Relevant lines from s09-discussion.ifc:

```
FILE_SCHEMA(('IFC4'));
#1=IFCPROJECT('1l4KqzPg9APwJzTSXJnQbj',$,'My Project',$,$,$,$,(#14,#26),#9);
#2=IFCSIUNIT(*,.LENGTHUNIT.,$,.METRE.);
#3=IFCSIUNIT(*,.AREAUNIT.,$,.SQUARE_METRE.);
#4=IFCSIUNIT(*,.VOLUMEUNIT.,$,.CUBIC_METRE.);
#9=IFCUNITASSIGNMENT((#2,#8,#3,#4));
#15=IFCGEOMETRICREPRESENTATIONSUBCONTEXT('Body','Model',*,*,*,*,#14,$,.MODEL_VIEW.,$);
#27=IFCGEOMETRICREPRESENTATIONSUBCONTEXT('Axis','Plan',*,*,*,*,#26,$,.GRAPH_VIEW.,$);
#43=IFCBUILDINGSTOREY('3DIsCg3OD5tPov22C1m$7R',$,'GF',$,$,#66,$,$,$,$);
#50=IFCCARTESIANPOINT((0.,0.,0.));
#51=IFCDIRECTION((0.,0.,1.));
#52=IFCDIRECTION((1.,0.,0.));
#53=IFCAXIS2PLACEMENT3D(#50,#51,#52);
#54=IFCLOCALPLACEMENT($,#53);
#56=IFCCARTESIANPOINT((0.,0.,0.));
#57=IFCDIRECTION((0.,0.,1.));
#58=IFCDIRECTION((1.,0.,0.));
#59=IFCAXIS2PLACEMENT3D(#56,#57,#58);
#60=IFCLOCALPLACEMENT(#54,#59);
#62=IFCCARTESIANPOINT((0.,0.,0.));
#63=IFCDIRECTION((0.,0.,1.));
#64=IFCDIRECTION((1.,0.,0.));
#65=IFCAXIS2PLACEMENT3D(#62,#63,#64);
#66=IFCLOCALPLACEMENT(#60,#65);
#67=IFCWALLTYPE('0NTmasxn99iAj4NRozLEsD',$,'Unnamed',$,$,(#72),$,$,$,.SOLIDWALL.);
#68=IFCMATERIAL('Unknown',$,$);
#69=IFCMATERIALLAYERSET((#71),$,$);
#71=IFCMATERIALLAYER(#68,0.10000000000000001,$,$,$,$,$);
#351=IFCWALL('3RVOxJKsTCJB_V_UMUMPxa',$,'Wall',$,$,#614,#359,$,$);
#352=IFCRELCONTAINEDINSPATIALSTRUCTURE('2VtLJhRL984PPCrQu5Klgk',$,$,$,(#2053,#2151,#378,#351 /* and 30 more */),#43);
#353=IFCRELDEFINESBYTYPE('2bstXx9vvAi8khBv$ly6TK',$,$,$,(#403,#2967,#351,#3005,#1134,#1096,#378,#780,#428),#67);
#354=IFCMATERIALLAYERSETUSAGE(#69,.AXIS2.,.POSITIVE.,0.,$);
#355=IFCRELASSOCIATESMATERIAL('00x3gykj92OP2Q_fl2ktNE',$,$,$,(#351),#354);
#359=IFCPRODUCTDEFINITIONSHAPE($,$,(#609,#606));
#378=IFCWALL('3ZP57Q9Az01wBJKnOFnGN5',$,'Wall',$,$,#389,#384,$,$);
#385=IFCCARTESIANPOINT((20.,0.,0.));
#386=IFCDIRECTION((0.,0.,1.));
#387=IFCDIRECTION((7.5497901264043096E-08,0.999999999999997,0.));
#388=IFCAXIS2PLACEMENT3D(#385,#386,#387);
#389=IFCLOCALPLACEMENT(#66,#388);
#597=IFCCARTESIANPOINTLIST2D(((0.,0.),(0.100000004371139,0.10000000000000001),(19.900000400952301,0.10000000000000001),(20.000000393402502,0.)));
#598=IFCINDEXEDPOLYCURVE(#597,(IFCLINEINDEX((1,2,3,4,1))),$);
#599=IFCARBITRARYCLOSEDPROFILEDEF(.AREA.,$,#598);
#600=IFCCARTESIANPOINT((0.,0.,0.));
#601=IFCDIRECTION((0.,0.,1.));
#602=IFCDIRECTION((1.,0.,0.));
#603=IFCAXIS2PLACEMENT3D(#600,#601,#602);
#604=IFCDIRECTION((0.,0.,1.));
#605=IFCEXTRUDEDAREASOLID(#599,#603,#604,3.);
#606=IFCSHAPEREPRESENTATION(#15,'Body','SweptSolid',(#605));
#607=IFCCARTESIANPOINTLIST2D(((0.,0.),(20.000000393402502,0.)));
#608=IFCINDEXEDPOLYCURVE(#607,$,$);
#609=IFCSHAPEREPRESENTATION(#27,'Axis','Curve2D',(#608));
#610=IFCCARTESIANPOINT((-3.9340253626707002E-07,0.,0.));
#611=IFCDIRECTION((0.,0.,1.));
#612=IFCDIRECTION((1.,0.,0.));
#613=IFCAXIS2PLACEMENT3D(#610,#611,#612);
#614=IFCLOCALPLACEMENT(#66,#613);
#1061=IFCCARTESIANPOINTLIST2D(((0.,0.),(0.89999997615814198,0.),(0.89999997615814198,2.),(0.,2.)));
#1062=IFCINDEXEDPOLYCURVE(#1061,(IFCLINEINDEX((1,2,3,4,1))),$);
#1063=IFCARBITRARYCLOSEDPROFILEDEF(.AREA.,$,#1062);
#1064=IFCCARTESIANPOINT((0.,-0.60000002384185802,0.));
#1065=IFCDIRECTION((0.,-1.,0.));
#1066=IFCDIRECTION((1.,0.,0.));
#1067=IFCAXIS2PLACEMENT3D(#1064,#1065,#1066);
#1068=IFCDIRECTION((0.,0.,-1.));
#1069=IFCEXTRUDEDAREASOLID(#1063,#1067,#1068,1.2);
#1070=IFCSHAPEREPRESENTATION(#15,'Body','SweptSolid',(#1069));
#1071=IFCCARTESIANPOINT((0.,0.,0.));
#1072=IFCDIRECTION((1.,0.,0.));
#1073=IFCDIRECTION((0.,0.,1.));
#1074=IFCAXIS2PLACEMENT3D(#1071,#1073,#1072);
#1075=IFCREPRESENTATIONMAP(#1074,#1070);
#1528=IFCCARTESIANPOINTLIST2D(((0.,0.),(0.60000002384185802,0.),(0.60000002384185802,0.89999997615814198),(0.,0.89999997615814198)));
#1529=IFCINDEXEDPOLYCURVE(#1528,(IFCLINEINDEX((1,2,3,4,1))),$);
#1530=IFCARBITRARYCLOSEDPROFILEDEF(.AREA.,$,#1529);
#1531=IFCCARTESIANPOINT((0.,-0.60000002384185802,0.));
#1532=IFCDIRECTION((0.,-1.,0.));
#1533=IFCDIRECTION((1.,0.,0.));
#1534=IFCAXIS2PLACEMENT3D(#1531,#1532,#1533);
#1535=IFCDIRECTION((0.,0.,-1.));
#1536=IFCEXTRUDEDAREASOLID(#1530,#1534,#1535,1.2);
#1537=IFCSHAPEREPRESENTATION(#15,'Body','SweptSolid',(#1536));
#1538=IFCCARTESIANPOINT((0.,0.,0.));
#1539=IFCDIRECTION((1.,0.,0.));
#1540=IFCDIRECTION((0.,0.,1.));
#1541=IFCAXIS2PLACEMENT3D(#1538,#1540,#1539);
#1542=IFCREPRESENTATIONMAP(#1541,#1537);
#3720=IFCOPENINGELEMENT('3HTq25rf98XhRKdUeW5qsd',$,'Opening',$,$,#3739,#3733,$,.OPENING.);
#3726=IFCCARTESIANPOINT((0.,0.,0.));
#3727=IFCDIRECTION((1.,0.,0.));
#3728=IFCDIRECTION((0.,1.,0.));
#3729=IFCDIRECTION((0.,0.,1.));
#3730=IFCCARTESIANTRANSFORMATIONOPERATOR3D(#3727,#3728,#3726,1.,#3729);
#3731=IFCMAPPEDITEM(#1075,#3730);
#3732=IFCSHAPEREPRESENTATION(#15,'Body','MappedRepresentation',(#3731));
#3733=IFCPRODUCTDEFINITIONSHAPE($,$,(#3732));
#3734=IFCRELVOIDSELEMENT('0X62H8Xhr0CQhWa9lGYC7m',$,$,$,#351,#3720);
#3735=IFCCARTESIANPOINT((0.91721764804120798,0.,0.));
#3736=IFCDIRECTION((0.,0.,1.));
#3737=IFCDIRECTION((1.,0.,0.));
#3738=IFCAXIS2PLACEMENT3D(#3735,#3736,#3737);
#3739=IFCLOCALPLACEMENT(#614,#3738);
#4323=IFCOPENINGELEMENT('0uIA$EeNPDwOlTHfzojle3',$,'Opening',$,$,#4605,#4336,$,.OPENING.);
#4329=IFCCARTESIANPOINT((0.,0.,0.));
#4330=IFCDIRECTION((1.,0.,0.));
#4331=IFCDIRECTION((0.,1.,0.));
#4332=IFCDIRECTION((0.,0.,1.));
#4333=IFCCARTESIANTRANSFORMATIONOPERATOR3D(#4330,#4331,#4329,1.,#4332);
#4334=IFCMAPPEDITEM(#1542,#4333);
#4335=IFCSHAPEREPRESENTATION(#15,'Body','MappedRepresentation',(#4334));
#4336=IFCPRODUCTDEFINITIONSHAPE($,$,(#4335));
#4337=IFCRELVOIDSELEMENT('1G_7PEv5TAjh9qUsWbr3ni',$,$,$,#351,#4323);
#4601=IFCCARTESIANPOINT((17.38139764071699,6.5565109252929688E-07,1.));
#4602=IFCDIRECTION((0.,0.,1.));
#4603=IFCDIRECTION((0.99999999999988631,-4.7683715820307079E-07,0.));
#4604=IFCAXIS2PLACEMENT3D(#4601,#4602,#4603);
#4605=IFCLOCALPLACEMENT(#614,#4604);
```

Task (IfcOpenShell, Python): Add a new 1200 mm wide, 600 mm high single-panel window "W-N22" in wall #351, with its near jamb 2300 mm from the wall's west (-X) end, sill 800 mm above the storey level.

```python
import numpy as np
import ifcopenshell
import ifcopenshell.api.feature
import ifcopenshell.api.geometry
import ifcopenshell.api.root
import ifcopenshell.api.spatial
import ifcopenshell.geom
import ifcopenshell.util.element
import ifcopenshell.util.placement
import ifcopenshell.util.representation
import ifcopenshell.util.shape
import ifcopenshell.util.unit

model = ifcopenshell.open("s09-discussion.ifc")
unit_scale = ifcopenshell.util.unit.calculate_unit_scale(model)
settings = ifcopenshell.geom.settings()


def volume(element):
    """Net volume in cubic metres, openings subtracted."""
    shape = ifcopenshell.geom.create_shape(settings, element)
    return ifcopenshell.util.shape.get_volume(shape.geometry)


wall = model.by_id(351)
storey = ifcopenshell.util.element.get_container(wall, ifc_class="IfcBuildingStorey")
context = ifcopenshell.util.representation.get_context(model, "Model", "Body", "MODEL_VIEW")
before = volume(wall)

width, height, from_end, sill = 1.2, 0.6, 2.3, 0.8  # metres

# The wall runs along its own X axis, and the end named is its -X end.
wall_shape = ifcopenshell.geom.create_shape(settings, wall)
x, y, z = ifcopenshell.util.shape.get_vertices(wall_shape.geometry).T
start = x.min() + from_end
face, thickness = float(y.min()), float(y.max() - y.min())
wall_matrix = ifcopenshell.util.placement.get_local_placement(wall.ObjectPlacement)
level = ifcopenshell.util.placement.get_local_placement(storey.ObjectPlacement)[2, 3]


def in_wall(x, y):
    """Placement at x, y metres in the wall's axes, at sill height."""
    matrix = wall_matrix.copy()
    matrix[:, 3] = wall_matrix @ np.array([x / unit_scale, y / unit_scale, 0.0, 1.0])
    matrix[2, 3] = level + sill / unit_scale
    return matrix


# Opening: a box that overshoots both wall faces by 50 mm.
opening = ifcopenshell.api.root.create_entity(model, ifc_class="IfcOpeningElement", predefined_type="OPENING")
box = ifcopenshell.api.geometry.add_wall_representation(
    model, context=context, length=width, height=height, thickness=thickness + 0.1
)
ifcopenshell.api.geometry.assign_representation(model, product=opening, representation=box)
ifcopenshell.api.geometry.edit_object_placement(model, product=opening, matrix=in_wall(start, face - 0.05), is_si=False)
ifcopenshell.api.feature.add_feature(model, feature=opening, element=wall)

window = ifcopenshell.api.root.create_entity(model, ifc_class="IfcWindow", name="W-N22", predefined_type="WINDOW")
window.OverallWidth, window.OverallHeight = width / unit_scale, height / unit_scale
window.PartitioningType = "SINGLE_PANEL"
body = ifcopenshell.api.geometry.add_window_representation(
    model,
    context=context,
    overall_width=window.OverallWidth,
    overall_height=window.OverallHeight,
    partition_type="SINGLE_PANEL",
)
ifcopenshell.api.geometry.assign_representation(model, product=window, representation=body)
ifcopenshell.api.spatial.assign_container(model, products=[window], relating_structure=storey)
ifcopenshell.api.feature.add_filling(model, opening=opening, element=window)

# Centre the window in the wall's thickness.
ifcopenshell.api.geometry.edit_object_placement(model, product=window, matrix=in_wall(start, face), is_si=False)
window_shape = ifcopenshell.geom.create_shape(settings, window)
depth = ifcopenshell.util.shape.get_vertices(window_shape.geometry)[:, 1]
offset = face + thickness / 2 - (depth.min() + depth.max()) / 2
ifcopenshell.api.geometry.edit_object_placement(model, product=window, matrix=in_wall(start, offset), is_si=False)

after = volume(wall)

print(f"wall volume {before:.3f} -> {after:.3f} m3")

model.write("s09-discussion_updated.ifc")
```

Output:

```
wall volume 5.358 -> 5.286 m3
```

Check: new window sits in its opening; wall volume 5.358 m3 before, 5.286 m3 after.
